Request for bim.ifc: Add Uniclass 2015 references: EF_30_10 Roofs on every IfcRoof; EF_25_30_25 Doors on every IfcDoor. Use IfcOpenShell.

First a look at what the model holds.

```python
import ifcopenshell

model = ifcopenshell.open("bim.ifc")
print(model.schema)
print("classifications:", [c.Name for c in model.by_type("IfcClassification")])
for ifc_class in ("IfcDoor", "IfcRoof", "IfcStair", "IfcWall", "IfcWindow"):
    print(ifc_class, len(model.by_type(ifc_class)))
```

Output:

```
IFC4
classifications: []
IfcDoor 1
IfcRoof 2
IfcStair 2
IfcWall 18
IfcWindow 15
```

```python
import ifcopenshell
import ifcopenshell.api.classification

model = ifcopenshell.open("bim.ifc")

system = ifcopenshell.api.classification.add_classification(model, classification="Uniclass 2015")

codes = {
    "IfcRoof": ("EF_30_10", "Roofs"),
    "IfcDoor": ("EF_25_30_25", "Doors"),
}
for ifc_class, (code, name) in codes.items():
    products = model.by_type(ifc_class)
    ifcopenshell.api.classification.add_reference(
        model, products=products, classification=system, identification=code, name=name
    )
    print(code, len(products))

model.write("bim_v2.ifc")
```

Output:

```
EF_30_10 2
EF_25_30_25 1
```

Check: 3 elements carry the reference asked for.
